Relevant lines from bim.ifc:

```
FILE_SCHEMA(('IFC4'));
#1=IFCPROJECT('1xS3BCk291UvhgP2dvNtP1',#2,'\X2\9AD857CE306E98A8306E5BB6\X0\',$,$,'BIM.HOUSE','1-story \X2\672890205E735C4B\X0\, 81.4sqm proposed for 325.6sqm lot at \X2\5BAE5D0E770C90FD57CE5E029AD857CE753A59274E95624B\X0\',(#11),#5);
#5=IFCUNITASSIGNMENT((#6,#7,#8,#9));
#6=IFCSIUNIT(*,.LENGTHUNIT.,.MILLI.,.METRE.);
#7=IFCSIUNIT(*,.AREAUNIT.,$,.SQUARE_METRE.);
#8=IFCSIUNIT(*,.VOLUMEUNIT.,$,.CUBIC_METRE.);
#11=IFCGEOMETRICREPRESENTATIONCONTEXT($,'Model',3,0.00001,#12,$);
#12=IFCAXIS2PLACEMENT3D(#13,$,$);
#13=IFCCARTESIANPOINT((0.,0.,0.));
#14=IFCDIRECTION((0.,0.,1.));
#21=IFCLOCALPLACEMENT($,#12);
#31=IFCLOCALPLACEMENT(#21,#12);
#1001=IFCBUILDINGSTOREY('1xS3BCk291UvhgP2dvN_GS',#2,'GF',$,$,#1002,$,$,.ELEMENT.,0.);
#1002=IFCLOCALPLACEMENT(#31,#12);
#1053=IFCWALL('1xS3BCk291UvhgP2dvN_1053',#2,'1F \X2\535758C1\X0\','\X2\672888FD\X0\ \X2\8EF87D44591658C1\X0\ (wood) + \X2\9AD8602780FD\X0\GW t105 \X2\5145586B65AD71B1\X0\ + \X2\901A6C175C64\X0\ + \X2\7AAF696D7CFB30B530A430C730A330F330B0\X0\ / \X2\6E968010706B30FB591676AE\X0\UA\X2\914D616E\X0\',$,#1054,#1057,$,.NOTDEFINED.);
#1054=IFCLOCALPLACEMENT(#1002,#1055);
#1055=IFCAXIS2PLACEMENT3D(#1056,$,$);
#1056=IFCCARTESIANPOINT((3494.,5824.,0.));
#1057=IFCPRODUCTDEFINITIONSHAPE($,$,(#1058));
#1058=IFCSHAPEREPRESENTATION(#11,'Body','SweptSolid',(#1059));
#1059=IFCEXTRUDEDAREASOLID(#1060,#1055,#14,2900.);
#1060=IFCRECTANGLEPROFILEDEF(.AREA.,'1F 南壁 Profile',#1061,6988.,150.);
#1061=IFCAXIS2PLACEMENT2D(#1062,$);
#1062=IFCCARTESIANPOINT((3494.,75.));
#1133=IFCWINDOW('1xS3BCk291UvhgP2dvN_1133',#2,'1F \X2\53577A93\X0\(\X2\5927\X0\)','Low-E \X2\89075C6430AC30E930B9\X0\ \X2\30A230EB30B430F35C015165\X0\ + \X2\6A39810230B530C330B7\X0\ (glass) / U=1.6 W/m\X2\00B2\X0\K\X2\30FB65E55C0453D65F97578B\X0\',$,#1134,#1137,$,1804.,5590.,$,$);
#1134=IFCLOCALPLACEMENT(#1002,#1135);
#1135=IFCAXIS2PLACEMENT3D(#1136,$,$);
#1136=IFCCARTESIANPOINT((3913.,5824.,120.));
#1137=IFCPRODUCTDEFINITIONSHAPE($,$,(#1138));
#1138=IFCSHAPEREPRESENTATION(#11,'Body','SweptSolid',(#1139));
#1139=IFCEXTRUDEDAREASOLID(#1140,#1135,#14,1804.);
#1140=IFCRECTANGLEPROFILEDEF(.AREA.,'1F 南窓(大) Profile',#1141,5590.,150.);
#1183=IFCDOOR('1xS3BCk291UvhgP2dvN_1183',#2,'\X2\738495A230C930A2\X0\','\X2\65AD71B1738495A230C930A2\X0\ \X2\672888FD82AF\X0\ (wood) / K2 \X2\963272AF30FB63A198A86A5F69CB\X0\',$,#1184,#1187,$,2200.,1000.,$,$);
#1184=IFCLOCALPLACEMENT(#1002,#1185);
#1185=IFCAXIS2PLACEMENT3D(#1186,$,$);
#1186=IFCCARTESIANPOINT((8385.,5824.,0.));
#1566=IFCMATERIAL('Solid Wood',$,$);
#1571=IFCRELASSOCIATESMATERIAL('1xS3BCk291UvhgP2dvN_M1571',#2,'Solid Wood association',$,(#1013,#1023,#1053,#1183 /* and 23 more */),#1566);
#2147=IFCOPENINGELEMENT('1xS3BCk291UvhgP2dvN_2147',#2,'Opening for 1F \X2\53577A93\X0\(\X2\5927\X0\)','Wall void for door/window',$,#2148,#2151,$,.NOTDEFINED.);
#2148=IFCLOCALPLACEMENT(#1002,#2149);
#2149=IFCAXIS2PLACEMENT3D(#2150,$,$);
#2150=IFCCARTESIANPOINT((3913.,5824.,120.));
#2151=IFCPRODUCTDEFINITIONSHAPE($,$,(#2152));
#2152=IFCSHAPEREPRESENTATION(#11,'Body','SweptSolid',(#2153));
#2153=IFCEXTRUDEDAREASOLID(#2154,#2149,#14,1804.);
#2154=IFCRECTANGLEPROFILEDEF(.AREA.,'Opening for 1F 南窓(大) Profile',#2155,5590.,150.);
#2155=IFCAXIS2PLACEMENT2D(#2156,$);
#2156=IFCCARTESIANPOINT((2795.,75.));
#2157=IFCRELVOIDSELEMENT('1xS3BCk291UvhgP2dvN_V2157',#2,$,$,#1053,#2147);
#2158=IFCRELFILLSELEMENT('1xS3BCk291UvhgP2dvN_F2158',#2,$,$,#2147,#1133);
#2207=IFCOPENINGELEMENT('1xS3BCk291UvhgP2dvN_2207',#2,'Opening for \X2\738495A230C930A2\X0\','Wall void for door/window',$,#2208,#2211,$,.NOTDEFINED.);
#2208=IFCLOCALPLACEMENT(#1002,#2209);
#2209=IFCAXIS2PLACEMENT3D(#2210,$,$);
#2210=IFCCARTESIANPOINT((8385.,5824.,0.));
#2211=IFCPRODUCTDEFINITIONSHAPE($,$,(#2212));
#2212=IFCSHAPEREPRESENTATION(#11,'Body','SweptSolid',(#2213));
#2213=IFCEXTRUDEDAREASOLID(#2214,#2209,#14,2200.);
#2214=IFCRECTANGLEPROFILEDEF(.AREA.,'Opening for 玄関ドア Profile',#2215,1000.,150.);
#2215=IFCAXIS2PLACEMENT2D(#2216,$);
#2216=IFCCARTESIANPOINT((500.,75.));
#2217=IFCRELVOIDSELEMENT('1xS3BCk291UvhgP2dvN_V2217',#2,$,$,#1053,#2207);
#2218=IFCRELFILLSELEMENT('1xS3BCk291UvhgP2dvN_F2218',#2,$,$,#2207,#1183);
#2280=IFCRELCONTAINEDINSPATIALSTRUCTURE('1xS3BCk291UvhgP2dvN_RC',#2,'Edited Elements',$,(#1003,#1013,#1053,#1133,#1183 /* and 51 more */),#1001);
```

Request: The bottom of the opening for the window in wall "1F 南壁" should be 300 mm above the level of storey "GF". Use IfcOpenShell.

```python
import numpy as np
import ifcopenshell
import ifcopenshell.api.geometry
import ifcopenshell.geom
import ifcopenshell.util.element
import ifcopenshell.util.placement
import ifcopenshell.util.shape
import ifcopenshell.util.unit

model = ifcopenshell.open("bim.ifc")
unit_scale = ifcopenshell.util.unit.calculate_unit_scale(model)

window = model.by_guid("1xS3BCk291UvhgP2dvN_1133")
opening = window.FillsVoids[0].RelatingOpeningElement
storey = ifcopenshell.util.element.get_container(window, ifc_class="IfcBuildingStorey")
level = ifcopenshell.util.placement.get_local_placement(storey.ObjectPlacement)[2, 3]

# The opening's origin need not be at the sill, so measure its lowest point.
shape = ifcopenshell.geom.create_shape(ifcopenshell.geom.settings(), opening)
bottom = ifcopenshell.util.shape.get_shape_bottom_elevation(shape, shape.geometry) / unit_scale
dz = level + 0.3 / unit_scale - bottom

shift = np.array([0.0, 0.0, dz])
# The window is not placed relative to its opening, so move both.
for product in (opening, window):
    matrix = ifcopenshell.util.placement.get_local_placement(product.ObjectPlacement)
    matrix[:3, 3] += shift
    ifcopenshell.api.geometry.edit_object_placement(model, product=product, matrix=matrix, is_si=False)

print(f"moved by {dz * unit_scale:+.3f} m")

model.write("bim_updated.ifc")
```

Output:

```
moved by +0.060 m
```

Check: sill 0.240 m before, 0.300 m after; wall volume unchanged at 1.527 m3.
